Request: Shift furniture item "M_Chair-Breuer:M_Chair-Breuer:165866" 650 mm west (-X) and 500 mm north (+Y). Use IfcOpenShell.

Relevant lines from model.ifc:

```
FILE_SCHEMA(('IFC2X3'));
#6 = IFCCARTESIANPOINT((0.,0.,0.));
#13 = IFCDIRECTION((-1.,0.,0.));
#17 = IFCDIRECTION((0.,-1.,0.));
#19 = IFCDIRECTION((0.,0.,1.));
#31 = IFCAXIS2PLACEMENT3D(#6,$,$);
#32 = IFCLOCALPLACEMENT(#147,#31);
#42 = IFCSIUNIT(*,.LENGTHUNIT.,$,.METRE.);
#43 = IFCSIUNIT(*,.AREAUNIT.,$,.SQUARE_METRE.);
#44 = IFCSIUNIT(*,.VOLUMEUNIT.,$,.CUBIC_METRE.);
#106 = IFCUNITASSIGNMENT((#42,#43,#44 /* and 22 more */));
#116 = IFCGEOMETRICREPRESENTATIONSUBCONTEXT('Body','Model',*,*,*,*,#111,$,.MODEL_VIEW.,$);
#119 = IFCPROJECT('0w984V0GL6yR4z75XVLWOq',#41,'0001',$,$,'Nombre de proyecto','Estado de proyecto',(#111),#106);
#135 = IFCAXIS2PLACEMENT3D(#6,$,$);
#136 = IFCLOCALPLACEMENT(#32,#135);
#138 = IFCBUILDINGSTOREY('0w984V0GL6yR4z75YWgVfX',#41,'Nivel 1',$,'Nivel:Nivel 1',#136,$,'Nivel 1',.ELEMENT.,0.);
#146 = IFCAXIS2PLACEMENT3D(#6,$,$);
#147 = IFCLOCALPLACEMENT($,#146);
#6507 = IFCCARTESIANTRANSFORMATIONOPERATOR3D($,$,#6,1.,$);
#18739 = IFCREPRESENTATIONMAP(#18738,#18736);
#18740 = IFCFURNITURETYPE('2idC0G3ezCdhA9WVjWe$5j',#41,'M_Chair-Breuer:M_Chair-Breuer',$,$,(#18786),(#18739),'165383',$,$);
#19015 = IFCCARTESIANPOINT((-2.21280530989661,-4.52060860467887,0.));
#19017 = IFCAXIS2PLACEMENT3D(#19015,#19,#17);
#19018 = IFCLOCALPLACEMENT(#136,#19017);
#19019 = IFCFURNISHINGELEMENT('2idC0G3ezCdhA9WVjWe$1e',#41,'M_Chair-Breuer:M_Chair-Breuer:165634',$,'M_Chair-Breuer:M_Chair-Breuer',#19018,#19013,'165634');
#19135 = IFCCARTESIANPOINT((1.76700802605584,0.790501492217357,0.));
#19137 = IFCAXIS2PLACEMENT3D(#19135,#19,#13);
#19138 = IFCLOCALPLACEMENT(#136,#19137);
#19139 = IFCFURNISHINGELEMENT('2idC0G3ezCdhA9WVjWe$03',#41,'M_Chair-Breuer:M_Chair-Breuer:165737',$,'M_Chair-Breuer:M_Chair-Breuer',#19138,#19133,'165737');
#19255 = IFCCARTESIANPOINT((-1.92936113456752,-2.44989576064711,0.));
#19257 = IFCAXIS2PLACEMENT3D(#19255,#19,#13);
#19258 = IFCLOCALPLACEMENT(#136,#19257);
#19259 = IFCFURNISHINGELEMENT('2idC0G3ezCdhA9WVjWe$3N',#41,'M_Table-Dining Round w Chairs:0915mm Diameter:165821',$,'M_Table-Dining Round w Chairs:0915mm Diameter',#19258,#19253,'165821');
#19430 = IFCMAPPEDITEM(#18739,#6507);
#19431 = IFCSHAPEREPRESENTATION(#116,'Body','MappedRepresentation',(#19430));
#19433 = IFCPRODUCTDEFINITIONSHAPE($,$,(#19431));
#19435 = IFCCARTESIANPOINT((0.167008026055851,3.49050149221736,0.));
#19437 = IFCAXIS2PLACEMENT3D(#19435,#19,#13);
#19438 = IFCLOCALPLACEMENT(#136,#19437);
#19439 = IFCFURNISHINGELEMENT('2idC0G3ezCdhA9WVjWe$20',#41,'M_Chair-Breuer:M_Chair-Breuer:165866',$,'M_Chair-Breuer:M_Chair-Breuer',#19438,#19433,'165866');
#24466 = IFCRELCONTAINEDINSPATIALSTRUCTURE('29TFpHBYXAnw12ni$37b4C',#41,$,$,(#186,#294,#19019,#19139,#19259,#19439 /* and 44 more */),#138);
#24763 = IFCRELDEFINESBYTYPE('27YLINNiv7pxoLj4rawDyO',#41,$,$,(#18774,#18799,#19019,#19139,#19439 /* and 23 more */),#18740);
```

```python
import ifcopenshell
import ifcopenshell.api.geometry
import ifcopenshell.util.placement
import ifcopenshell.util.unit

model = ifcopenshell.open("model.ifc")
unit_scale = ifcopenshell.util.unit.calculate_unit_scale(model)

item = model.by_guid("2idC0G3ezCdhA9WVjWe$20")
matrix = ifcopenshell.util.placement.get_local_placement(item.ObjectPlacement)
matrix[0, 3] -= 0.65 / unit_scale
matrix[1, 3] += 0.5 / unit_scale
ifcopenshell.api.geometry.edit_object_placement(model, product=item, matrix=matrix, is_si=False)

print(ifcopenshell.util.placement.get_local_placement(item.ObjectPlacement).round(3) + 0.0)

model.write("model_updated.ifc")
```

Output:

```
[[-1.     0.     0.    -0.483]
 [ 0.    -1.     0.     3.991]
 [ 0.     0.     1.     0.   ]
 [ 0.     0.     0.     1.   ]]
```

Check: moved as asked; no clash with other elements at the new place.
